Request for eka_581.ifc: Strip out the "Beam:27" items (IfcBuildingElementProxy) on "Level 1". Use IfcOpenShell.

First a look at what the model holds.

```python
import ifcopenshell
import ifcopenshell.util.element

model = ifcopenshell.open("eka_581.ifc")
print(model.schema)
storey = next(s for s in model.by_type("IfcBuildingStorey") if s.Name == "Level 1")
proxies = [e for e in ifcopenshell.util.element.get_decomposition(storey) if e.is_a("IfcBuildingElementProxy")]
seen = {}
for e in proxies:
    element_type = ifcopenshell.util.element.get_type(e)
    name = element_type.Name if element_type not in (None, e) else None
    seen[name] = seen.get(name, 0) + 1
for name, count in sorted(seen.items(), key=str):
    print(count, "x", name)
```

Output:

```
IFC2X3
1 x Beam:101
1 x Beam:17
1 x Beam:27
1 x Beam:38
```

```python
import ifcopenshell
import ifcopenshell.api.root
import ifcopenshell.util.element

model = ifcopenshell.open("eka_581.ifc")

storey = next(s for s in model.by_type("IfcBuildingStorey") if s.Name == "Level 1")
proxies = [e for e in ifcopenshell.util.element.get_decomposition(storey) if e.is_a("IfcBuildingElementProxy")]
targets = [e for e in proxies if (t := ifcopenshell.util.element.get_type(e)) not in (None, e) and t.Name == "Beam:27"]

for e in targets:
    ifcopenshell.api.root.remove_product(model, product=e)
print(len(targets), "removed")

model.write("eka_581_updated.ifc")
```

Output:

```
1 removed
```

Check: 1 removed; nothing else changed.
